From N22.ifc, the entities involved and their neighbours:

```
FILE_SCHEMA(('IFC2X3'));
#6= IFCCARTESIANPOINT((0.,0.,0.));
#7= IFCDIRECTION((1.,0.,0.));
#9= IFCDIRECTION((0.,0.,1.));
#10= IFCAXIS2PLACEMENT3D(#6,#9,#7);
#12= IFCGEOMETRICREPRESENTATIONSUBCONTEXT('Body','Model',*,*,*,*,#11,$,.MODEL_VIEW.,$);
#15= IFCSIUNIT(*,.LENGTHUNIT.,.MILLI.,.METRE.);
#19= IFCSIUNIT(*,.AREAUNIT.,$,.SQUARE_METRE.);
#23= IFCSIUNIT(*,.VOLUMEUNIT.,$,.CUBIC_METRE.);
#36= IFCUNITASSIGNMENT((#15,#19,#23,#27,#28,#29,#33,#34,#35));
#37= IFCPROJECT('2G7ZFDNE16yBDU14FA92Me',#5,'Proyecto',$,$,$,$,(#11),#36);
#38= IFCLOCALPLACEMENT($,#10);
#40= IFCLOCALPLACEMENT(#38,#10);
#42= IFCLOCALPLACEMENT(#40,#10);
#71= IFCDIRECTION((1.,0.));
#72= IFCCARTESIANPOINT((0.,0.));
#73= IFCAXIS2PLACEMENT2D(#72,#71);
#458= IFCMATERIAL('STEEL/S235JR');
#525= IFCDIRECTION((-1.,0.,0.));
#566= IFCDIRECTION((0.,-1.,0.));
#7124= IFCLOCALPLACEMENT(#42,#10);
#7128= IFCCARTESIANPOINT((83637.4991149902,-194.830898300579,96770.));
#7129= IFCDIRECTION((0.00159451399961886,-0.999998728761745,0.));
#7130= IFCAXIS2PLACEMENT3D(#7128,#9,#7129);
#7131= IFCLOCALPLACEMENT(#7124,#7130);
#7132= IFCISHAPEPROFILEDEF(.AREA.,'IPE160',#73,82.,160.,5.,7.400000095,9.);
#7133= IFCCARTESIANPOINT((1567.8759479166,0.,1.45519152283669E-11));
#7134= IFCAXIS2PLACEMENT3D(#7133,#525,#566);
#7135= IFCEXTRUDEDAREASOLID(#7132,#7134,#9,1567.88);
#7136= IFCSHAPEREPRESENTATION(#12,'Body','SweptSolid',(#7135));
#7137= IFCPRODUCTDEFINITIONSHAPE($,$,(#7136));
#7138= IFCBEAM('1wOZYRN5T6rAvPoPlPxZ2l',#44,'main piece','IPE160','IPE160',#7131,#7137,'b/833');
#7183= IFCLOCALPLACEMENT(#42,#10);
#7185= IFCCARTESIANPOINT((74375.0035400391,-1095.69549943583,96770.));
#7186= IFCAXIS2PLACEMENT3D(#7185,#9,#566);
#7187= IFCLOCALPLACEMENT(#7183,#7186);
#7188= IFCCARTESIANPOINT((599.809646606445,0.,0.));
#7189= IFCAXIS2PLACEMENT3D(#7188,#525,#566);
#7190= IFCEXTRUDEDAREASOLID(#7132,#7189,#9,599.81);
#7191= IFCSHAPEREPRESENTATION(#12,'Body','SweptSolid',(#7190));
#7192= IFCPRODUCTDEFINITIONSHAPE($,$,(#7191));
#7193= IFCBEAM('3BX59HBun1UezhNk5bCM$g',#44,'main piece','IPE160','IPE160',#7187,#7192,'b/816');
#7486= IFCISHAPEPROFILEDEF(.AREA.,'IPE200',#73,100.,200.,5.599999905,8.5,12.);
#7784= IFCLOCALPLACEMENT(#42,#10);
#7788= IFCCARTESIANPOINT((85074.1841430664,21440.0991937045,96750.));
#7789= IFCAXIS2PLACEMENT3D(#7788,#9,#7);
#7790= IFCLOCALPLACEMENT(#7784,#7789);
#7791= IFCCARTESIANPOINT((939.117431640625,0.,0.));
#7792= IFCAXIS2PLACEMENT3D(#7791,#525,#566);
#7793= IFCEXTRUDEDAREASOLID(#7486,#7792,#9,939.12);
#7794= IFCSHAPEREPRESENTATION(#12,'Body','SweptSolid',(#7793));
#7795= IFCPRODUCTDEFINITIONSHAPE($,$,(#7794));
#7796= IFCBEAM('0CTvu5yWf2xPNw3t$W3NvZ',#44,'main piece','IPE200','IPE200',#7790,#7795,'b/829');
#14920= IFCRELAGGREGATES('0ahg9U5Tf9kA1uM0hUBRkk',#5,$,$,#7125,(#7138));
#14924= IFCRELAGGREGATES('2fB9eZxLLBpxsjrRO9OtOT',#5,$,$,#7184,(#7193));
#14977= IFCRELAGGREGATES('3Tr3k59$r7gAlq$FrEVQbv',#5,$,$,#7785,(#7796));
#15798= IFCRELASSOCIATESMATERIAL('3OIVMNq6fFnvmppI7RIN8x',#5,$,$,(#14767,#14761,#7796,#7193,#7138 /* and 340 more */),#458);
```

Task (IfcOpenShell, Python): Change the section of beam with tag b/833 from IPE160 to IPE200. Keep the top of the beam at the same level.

```python
import ifcopenshell
import ifcopenshell.util.element
import ifcopenshell.util.representation

model = ifcopenshell.open("N22.ifc")

member = model.by_id(7138)
source = next(p for p in model.by_type("IfcIShapeProfileDef") if p.ProfileName == "IPE200")

body = ifcopenshell.util.representation.get_representation(member, "Model", "Body")
solid = body.Items[0]
old_profile = solid.SweptArea

# Copy the section's sizes but keep this member's own profile position.
profile = ifcopenshell.util.element.copy(model, source)
# Profiles are centred, so shift by half the change in depth to hold the top.
shift = (old_profile.OverallDepth - profile.OverallDepth) / 2
x, y = old_profile.Position.Location.Coordinates
up = (0.0, 1.0)  # upwards, in the solid's own plane
location = model.createIfcCartesianPoint((x + up[0] * shift, y + up[1] * shift))
profile.Position = model.createIfcAxis2Placement2D(location, old_profile.Position.RefDirection)
solid.SweptArea = profile
if not model.get_total_inverses(old_profile):
    ifcopenshell.util.element.remove_deep2(model, old_profile)
member.Description = member.Description.replace("IPE160", "IPE200")
member.ObjectType = member.ObjectType.replace("IPE160", "IPE200")

print(solid.SweptArea)

model.write("N22-out.ifc")
```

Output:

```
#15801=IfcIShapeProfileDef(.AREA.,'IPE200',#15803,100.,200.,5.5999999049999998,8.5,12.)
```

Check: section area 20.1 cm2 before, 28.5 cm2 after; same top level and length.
